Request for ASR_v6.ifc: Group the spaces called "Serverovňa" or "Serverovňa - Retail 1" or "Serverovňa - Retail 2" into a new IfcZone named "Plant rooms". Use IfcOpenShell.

First a look at what the model holds.

```python
import ifcopenshell

model = ifcopenshell.open("ASR_v6.ifc")
print(model.schema)
seen = {}
for space in model.by_type("IfcSpace"):
    seen[space.LongName] = seen.get(space.LongName, 0) + 1
for name, count in sorted(seen.items(), key=str):
    print(count, "x", name)
print("zones:", [z.Name for z in model.by_type("IfcZone")][:20])
```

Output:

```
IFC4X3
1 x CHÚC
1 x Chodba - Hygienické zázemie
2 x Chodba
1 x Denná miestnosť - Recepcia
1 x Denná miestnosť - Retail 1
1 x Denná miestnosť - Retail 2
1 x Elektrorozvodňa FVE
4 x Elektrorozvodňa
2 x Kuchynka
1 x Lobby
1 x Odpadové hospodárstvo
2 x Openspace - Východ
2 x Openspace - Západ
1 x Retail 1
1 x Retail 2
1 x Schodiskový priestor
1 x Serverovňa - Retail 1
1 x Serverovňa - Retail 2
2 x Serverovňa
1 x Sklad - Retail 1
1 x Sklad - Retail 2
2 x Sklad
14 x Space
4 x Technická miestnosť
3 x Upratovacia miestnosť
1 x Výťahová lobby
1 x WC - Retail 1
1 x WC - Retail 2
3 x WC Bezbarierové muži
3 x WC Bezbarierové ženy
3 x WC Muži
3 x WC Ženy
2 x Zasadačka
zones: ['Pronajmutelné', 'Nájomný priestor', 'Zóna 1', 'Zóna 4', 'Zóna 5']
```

```python
import ifcopenshell
import ifcopenshell.api.group
import ifcopenshell.api.root

model = ifcopenshell.open("ASR_v6.ifc")

names = {"Serverovňa", "Serverovňa - Retail 1", "Serverovňa - Retail 2"}
spaces = [s for s in model.by_type("IfcSpace") if s.LongName in names]

zone = ifcopenshell.api.root.create_entity(model, ifc_class="IfcZone", name="Plant rooms")
ifcopenshell.api.group.assign_group(model, products=spaces, group=zone)
print(len(spaces), "spaces in", zone.Name)

model.write("ASR_v6_v2.ifc")
```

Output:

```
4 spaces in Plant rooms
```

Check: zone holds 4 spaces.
